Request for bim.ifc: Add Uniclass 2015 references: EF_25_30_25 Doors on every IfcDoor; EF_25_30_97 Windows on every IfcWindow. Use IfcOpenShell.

First a look at what the model holds.

```python
import ifcopenshell

model = ifcopenshell.open("bim.ifc")
print(model.schema)
print("classifications:", [c.Name for c in model.by_type("IfcClassification")])
for ifc_class in ("IfcDoor", "IfcRoof", "IfcStair", "IfcWall", "IfcWindow"):
    print(ifc_class, len(model.by_type(ifc_class)))
```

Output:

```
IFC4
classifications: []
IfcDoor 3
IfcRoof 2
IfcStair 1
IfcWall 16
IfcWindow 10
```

```python
import ifcopenshell
import ifcopenshell.api.classification

model = ifcopenshell.open("bim.ifc")

system = ifcopenshell.api.classification.add_classification(model, classification="Uniclass 2015")

codes = {
    "IfcDoor": ("EF_25_30_25", "Doors"),
    "IfcWindow": ("EF_25_30_97", "Windows"),
}
for ifc_class, (code, name) in codes.items():
    products = model.by_type(ifc_class)
    ifcopenshell.api.classification.add_reference(
        model, products=products, classification=system, identification=code, name=name
    )
    print(code, len(products))

model.write("bim_v2.ifc")
```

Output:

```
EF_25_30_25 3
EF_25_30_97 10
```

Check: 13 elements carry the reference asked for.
